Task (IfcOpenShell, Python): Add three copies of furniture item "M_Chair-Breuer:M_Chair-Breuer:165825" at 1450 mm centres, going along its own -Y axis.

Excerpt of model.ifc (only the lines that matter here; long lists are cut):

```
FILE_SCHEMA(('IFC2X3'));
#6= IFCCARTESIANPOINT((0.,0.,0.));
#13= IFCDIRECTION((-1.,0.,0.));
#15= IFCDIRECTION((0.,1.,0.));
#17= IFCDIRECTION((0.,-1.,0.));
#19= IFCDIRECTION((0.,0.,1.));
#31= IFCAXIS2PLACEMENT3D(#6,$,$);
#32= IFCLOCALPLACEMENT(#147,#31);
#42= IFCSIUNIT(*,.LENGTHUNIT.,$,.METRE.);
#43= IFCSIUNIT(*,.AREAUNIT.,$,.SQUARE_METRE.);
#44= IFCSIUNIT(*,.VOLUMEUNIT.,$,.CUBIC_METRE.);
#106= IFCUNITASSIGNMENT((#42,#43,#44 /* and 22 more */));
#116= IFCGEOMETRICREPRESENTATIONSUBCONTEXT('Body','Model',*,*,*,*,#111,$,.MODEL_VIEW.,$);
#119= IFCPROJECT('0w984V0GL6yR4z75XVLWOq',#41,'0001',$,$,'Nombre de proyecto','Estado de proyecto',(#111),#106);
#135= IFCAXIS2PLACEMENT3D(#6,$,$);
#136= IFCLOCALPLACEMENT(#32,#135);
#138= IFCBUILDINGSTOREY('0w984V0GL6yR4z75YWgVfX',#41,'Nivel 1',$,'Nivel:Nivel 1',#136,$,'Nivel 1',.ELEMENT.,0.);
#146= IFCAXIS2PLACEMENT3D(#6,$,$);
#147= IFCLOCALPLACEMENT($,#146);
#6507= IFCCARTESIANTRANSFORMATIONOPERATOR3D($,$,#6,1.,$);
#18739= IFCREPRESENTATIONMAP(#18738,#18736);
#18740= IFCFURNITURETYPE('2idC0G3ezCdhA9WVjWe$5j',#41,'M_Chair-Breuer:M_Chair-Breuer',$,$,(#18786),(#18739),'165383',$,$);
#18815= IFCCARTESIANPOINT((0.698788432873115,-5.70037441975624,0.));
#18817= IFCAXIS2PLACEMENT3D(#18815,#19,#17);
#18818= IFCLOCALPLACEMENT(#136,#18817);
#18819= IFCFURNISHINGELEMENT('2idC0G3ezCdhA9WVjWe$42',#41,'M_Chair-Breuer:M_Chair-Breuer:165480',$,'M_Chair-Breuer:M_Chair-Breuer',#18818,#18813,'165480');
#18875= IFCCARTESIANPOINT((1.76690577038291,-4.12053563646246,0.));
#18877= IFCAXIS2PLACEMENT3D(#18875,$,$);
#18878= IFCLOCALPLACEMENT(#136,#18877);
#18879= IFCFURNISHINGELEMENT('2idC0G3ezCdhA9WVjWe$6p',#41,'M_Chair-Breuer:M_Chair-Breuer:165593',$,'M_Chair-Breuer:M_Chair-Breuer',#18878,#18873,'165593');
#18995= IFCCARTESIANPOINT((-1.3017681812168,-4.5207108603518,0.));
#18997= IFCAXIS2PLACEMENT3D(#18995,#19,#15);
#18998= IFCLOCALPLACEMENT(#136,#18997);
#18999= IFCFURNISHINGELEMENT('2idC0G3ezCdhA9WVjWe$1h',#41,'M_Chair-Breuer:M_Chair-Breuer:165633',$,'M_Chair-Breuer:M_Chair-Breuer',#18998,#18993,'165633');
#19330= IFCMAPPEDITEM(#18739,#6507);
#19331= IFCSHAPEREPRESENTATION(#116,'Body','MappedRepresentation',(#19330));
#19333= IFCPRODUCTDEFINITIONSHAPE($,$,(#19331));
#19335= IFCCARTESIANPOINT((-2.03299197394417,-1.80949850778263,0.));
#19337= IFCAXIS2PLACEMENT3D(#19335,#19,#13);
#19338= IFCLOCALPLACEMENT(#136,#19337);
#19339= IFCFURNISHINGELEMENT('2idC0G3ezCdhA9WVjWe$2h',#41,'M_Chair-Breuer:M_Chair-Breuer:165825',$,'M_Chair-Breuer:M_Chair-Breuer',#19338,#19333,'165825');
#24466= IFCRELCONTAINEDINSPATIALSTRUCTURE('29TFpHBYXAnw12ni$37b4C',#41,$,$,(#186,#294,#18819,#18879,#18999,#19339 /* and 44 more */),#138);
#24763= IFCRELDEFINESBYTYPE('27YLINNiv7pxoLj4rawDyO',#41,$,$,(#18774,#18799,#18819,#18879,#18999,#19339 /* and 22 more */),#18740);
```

```python
import ifcopenshell
import ifcopenshell.api.geometry
import ifcopenshell.api.root
import ifcopenshell.util.element
import ifcopenshell.util.placement

model = ifcopenshell.open("model.ifc")


def reuse_history(source, copy):
    """copy_class also copies each property set's owner history, people and application; keep the originals."""
    for rel in copy.IsDefinedBy:
        if rel.is_a("IfcRelDefinesByProperties") and (history := rel.RelatingPropertyDefinition.OwnerHistory):
            rel.RelatingPropertyDefinition.OwnerHistory = source.OwnerHistory
            ifcopenshell.util.element.remove_deep2(model, history)


source = model.by_id(19339)
base = ifcopenshell.util.placement.get_local_placement(source.ObjectPlacement)
step = -base[:3, 1] * 1.45

for i in range(1, 4):
    copy = ifcopenshell.api.root.copy_class(model, product=source)
    copy.Representation = ifcopenshell.util.element.copy_deep(
        model, source.Representation, exclude=["IfcGeometricRepresentationContext", "IfcRepresentationMap"]
    )
    copy.Name = "M_Chair-Breuer:M_Chair-Breuer"
    copy.Tag = None
    reuse_history(source, copy)
    matrix = base.copy()
    matrix[:3, 3] += i * step
    print("added at", matrix[:3, 3].round(3) + 0.0)
    ifcopenshell.api.geometry.edit_object_placement(model, product=copy, matrix=matrix, is_si=False)

model.write("model_rev.ifc")
```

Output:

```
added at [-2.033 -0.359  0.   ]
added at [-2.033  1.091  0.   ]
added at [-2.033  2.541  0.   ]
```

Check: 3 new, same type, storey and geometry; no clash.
